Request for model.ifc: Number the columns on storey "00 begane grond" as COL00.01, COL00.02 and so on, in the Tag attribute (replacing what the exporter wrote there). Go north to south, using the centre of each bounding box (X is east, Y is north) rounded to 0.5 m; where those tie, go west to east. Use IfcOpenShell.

First a look at what the model holds.

```python
import ifcopenshell
import ifcopenshell.util.element
import ifcopenshell.util.placement

model = ifcopenshell.open("model.ifc")
print(model.schema)
storey = next(s for s in model.by_type("IfcBuildingStorey") if s.Name == "00 begane grond")
columns = [e for e in ifcopenshell.util.element.get_decomposition(storey) if e.is_a("IfcColumn")]
for e in sorted(columns, key=lambda e: e.id()):
    origin = ifcopenshell.util.placement.get_local_placement(e.ObjectPlacement)[:3, 3]
    print(e.id(), e.Tag, e.Name, origin.round(2) + 0.0, sep=" | ")
```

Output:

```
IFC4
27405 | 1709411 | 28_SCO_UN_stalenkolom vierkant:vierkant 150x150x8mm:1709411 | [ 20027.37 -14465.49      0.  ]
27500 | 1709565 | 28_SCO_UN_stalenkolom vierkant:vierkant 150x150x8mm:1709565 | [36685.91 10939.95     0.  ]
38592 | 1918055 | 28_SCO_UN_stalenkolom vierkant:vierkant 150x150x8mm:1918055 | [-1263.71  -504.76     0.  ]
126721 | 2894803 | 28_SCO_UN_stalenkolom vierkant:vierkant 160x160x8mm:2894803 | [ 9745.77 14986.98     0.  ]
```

```python
import ifcopenshell
import ifcopenshell.geom
import ifcopenshell.util.element
import ifcopenshell.util.shape

model = ifcopenshell.open("model.ifc")
settings = ifcopenshell.geom.settings()
settings.set("use-world-coords", True)


def centre(element):
    shape = ifcopenshell.geom.create_shape(settings, element)
    return ifcopenshell.util.shape.get_bbox_centroid(shape.geometry)


storey = next(s for s in model.by_type("IfcBuildingStorey") if s.Name == "00 begane grond")
columns = [e for e in ifcopenshell.util.element.get_decomposition(storey) if e.is_a("IfcColumn")]

# Insertion points can sit at a corner or the storey origin, so sort by the geometry (in metres).
centres = {e: centre(e) for e in columns}
columns.sort(key=lambda e: (-round(centres[e][1] / 0.5), centres[e][0]))

for i, e in enumerate(columns, start=1):
    number = f"COL00.{i:02d}"
    e.Tag = number
    print(e.id(), number)

model.write("model_edited.ifc")
```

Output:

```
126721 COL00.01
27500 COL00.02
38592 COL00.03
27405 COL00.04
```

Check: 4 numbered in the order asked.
